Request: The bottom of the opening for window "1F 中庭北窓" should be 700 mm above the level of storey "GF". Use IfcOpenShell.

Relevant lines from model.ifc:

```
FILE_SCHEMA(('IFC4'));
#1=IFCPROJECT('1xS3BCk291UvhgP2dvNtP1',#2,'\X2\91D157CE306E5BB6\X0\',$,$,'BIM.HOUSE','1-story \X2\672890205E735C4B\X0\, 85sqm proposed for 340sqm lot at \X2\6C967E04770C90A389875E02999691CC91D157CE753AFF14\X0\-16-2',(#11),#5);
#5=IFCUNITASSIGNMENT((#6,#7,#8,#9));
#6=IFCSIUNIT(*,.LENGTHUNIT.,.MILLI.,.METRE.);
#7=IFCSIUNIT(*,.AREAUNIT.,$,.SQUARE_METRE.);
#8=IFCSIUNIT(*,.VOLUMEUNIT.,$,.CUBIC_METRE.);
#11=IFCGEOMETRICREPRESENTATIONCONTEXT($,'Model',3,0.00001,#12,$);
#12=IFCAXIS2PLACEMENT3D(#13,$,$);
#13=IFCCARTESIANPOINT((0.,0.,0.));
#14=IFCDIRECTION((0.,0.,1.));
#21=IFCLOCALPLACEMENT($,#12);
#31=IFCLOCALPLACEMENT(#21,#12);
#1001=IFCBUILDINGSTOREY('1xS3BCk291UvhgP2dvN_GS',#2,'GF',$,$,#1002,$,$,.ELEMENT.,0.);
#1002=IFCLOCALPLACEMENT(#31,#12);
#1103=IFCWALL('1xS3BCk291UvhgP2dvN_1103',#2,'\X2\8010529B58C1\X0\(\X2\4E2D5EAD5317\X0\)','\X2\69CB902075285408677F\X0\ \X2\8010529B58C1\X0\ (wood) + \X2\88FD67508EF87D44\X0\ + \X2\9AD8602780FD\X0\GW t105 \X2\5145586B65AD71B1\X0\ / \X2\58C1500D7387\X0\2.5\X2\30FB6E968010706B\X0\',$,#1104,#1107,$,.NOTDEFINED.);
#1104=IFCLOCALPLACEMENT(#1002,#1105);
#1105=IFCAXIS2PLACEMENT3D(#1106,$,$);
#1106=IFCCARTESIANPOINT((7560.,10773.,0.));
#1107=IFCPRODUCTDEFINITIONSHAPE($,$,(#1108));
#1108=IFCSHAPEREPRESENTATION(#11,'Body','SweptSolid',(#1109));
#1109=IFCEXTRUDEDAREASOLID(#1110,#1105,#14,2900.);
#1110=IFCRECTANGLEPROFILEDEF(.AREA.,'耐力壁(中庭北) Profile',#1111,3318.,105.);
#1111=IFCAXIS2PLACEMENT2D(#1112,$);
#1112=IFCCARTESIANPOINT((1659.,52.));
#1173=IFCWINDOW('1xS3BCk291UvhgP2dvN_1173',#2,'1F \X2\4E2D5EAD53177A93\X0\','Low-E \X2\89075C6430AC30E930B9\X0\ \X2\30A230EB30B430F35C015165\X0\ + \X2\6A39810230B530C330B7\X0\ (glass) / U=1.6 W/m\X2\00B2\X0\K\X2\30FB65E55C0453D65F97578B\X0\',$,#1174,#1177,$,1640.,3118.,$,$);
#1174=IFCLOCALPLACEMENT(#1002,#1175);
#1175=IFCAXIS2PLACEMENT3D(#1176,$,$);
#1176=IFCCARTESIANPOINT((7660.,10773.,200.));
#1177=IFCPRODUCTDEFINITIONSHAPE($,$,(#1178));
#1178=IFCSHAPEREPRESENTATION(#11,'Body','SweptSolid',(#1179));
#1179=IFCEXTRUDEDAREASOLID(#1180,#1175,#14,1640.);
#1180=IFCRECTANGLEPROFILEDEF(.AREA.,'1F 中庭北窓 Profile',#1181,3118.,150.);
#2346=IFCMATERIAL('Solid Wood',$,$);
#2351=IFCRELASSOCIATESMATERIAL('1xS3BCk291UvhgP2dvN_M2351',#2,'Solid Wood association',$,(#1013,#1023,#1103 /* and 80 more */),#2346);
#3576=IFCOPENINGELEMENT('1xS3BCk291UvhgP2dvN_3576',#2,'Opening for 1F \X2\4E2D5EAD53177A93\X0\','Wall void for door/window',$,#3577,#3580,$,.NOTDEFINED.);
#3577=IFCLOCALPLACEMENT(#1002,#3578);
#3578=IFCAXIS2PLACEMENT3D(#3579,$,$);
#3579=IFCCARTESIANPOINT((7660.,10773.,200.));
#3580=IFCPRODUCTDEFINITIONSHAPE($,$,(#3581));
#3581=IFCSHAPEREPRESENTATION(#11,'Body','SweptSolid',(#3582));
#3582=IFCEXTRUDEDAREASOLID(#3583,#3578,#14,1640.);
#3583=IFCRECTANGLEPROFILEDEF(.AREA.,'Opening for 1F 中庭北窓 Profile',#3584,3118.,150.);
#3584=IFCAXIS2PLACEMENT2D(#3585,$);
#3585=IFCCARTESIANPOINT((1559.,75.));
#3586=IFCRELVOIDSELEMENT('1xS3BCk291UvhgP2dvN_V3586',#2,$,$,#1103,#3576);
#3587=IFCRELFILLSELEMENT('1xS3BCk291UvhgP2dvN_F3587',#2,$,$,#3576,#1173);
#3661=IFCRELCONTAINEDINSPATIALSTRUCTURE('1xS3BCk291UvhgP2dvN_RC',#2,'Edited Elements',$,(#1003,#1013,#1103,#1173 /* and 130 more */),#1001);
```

```python
import numpy as np
import ifcopenshell
import ifcopenshell.api.geometry
import ifcopenshell.geom
import ifcopenshell.util.element
import ifcopenshell.util.placement
import ifcopenshell.util.shape
import ifcopenshell.util.unit

model = ifcopenshell.open("model.ifc")
unit_scale = ifcopenshell.util.unit.calculate_unit_scale(model)

window = model.by_guid("1xS3BCk291UvhgP2dvN_1173")
opening = window.FillsVoids[0].RelatingOpeningElement
storey = ifcopenshell.util.element.get_container(window, ifc_class="IfcBuildingStorey")
level = ifcopenshell.util.placement.get_local_placement(storey.ObjectPlacement)[2, 3]

# The opening's origin need not be at the sill, so measure its lowest point.
shape = ifcopenshell.geom.create_shape(ifcopenshell.geom.settings(), opening)
bottom = ifcopenshell.util.shape.get_shape_bottom_elevation(shape, shape.geometry) / unit_scale
dz = level + 0.7 / unit_scale - bottom

shift = np.array([0.0, 0.0, dz])
# The window is not placed relative to its opening, so move both.
for product in (opening, window):
    matrix = ifcopenshell.util.placement.get_local_placement(product.ObjectPlacement)
    matrix[:3, 3] += shift
    ifcopenshell.api.geometry.edit_object_placement(model, product=product, matrix=matrix, is_si=False)

print(f"moved by {dz * unit_scale:+.3f} m")

model.write("model-out.ifc")
```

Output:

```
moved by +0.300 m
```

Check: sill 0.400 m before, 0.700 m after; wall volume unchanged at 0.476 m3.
